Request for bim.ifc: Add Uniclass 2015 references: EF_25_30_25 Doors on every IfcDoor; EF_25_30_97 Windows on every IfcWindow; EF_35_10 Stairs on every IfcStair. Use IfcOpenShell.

First a look at what the model holds.

```python
import ifcopenshell

model = ifcopenshell.open("bim.ifc")
print(model.schema)
print("classifications:", [c.Name for c in model.by_type("IfcClassification")])
for ifc_class in ("IfcDoor", "IfcRoof", "IfcStair", "IfcWall", "IfcWindow"):
    print(ifc_class, len(model.by_type(ifc_class)))
```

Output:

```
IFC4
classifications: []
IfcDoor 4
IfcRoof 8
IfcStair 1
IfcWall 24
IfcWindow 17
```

```python
import ifcopenshell
import ifcopenshell.api.classification

model = ifcopenshell.open("bim.ifc")

system = ifcopenshell.api.classification.add_classification(model, classification="Uniclass 2015")

codes = {
    "IfcDoor": ("EF_25_30_25", "Doors"),
    "IfcWindow": ("EF_25_30_97", "Windows"),
    "IfcStair": ("EF_35_10", "Stairs"),
}
for ifc_class, (code, name) in codes.items():
    products = model.by_type(ifc_class)
    ifcopenshell.api.classification.add_reference(
        model, products=products, classification=system, identification=code, name=name
    )
    print(code, len(products))

model.write("bim_v2.ifc")
```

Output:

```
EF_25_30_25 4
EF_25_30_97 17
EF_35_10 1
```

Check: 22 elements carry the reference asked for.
